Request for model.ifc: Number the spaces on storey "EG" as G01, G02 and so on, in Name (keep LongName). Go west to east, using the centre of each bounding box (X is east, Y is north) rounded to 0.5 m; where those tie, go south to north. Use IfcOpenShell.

First a look at what the model holds.

```python
import ifcopenshell
import ifcopenshell.util.element
import ifcopenshell.util.placement

model = ifcopenshell.open("model.ifc")
print(model.schema)
storey = next(s for s in model.by_type("IfcBuildingStorey") if s.Name == "EG")
spaces = [e for e in ifcopenshell.util.element.get_decomposition(storey) if e.is_a("IfcSpace")]
for e in sorted(spaces, key=lambda e: e.id()):
    origin = ifcopenshell.util.placement.get_local_placement(e.ObjectPlacement)[:3, 3]
    print(e.id(), e.Name, e.LongName, origin.round(2) + 0.0, sep=" | ")
```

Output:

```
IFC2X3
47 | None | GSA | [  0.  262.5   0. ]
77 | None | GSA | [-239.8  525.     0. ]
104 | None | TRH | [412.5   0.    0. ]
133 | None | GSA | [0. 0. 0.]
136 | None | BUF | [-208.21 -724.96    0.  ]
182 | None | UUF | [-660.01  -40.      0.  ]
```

```python
import ifcopenshell
import ifcopenshell.geom
import ifcopenshell.util.element
import ifcopenshell.util.shape

model = ifcopenshell.open("model.ifc")
settings = ifcopenshell.geom.settings()
settings.set("use-world-coords", True)


def centre(element):
    shape = ifcopenshell.geom.create_shape(settings, element)
    return ifcopenshell.util.shape.get_bbox_centroid(shape.geometry)


storey = next(s for s in model.by_type("IfcBuildingStorey") if s.Name == "EG")
spaces = [e for e in ifcopenshell.util.element.get_decomposition(storey) if e.is_a("IfcSpace")]

# Insertion points can sit at a corner or the storey origin, so sort by the geometry (in metres).
centres = {e: centre(e) for e in spaces}
spaces.sort(key=lambda e: (round(centres[e][0] / 0.5), centres[e][1]))

for i, e in enumerate(spaces, start=1):
    number = f"G{i:02d}"
    e.Name = number
    print(e.id(), number)

model.write("model_edited.ifc")
```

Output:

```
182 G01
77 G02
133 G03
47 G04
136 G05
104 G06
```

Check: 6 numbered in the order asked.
